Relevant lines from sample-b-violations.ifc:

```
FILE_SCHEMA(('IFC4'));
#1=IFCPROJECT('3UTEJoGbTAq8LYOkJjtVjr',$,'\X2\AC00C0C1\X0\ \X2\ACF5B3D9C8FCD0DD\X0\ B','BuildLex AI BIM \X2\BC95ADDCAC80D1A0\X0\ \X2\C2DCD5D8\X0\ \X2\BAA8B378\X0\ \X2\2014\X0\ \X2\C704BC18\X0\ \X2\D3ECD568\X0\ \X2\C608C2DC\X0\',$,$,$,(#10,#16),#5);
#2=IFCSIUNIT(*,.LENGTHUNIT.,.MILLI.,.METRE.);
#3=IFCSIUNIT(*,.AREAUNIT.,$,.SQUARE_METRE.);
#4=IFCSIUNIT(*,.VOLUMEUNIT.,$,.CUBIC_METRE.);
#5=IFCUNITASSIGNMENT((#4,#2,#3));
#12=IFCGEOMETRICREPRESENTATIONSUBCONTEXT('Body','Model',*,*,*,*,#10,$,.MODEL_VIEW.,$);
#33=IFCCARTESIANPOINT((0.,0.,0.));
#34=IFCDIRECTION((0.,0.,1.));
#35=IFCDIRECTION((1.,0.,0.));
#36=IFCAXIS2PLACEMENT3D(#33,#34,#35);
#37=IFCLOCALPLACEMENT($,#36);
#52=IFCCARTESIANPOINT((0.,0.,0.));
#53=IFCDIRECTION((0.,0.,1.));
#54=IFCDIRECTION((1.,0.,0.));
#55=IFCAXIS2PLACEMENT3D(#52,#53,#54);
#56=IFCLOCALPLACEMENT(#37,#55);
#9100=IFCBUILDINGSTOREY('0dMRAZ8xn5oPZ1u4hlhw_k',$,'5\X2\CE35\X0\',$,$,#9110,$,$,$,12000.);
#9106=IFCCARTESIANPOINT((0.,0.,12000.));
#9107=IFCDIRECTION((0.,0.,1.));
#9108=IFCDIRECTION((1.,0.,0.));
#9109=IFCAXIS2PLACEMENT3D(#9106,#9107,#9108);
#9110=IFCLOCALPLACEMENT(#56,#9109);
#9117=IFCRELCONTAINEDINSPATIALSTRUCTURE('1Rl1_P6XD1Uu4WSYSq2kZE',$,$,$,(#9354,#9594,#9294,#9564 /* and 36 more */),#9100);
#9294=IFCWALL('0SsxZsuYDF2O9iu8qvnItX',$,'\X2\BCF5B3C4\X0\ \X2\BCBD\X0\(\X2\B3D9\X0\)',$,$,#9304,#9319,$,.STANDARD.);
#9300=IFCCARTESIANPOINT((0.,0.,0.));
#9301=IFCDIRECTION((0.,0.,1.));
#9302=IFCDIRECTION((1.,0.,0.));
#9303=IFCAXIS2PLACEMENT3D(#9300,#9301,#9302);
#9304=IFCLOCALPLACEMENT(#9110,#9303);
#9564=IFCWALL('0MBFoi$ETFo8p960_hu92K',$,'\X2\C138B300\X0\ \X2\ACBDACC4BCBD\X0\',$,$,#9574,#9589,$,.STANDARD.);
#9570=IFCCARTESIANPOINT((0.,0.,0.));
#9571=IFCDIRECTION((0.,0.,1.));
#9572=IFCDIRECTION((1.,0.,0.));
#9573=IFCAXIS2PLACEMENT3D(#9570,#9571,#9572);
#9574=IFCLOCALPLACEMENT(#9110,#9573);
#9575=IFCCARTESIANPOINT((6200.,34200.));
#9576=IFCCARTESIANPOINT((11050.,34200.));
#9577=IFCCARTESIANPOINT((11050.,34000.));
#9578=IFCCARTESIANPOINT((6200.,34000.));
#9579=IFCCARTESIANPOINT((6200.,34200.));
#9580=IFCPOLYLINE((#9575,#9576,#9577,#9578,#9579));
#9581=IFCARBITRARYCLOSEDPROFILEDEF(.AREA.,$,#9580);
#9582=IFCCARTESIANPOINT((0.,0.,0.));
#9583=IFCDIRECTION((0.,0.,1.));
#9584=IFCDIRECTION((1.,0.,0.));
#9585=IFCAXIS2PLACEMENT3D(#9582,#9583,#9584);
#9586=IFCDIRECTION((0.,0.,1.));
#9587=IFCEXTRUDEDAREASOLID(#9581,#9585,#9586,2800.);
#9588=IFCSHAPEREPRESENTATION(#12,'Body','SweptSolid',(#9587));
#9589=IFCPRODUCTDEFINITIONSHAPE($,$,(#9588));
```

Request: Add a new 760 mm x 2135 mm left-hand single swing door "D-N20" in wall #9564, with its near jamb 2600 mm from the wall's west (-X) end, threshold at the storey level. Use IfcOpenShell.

```python
import numpy as np
import ifcopenshell
import ifcopenshell.api.feature
import ifcopenshell.api.geometry
import ifcopenshell.api.root
import ifcopenshell.api.spatial
import ifcopenshell.geom
import ifcopenshell.util.element
import ifcopenshell.util.placement
import ifcopenshell.util.representation
import ifcopenshell.util.shape
import ifcopenshell.util.unit

model = ifcopenshell.open("sample-b-violations.ifc")
unit_scale = ifcopenshell.util.unit.calculate_unit_scale(model)
settings = ifcopenshell.geom.settings()


def volume(element):
    """Net volume in cubic metres, openings subtracted."""
    shape = ifcopenshell.geom.create_shape(settings, element)
    return ifcopenshell.util.shape.get_volume(shape.geometry)


wall = model.by_guid("0MBFoi$ETFo8p960_hu92K")
storey = ifcopenshell.util.element.get_container(wall, ifc_class="IfcBuildingStorey")
context = ifcopenshell.util.representation.get_context(model, "Model", "Body", "MODEL_VIEW")
before = volume(wall)

width, height, from_end, sill = 0.76, 2.135, 2.6, 0.0  # metres

# The wall runs along its own X axis, and the end named is its -X end.
wall_shape = ifcopenshell.geom.create_shape(settings, wall)
x, y, z = ifcopenshell.util.shape.get_vertices(wall_shape.geometry).T
start = x.min() + from_end
face, thickness = float(y.min()), float(y.max() - y.min())
wall_matrix = ifcopenshell.util.placement.get_local_placement(wall.ObjectPlacement)
level = ifcopenshell.util.placement.get_local_placement(storey.ObjectPlacement)[2, 3]


def in_wall(x, y):
    """Placement at x, y metres in the wall's axes, at sill height."""
    matrix = wall_matrix.copy()
    matrix[:, 3] = wall_matrix @ np.array([x / unit_scale, y / unit_scale, 0.0, 1.0])
    matrix[2, 3] = level + sill / unit_scale
    return matrix


# Opening: a box that overshoots both wall faces by 50 mm.
opening = ifcopenshell.api.root.create_entity(model, ifc_class="IfcOpeningElement", predefined_type="OPENING")
box = ifcopenshell.api.geometry.add_wall_representation(
    model, context=context, length=width, height=height, thickness=thickness + 0.1
)
ifcopenshell.api.geometry.assign_representation(model, product=opening, representation=box)
ifcopenshell.api.geometry.edit_object_placement(model, product=opening, matrix=in_wall(start, face - 0.05), is_si=False)
ifcopenshell.api.feature.add_feature(model, feature=opening, element=wall)

door = ifcopenshell.api.root.create_entity(model, ifc_class="IfcDoor", name="D-N20", predefined_type="DOOR")
door.OverallWidth, door.OverallHeight = width / unit_scale, height / unit_scale
door.OperationType = "SINGLE_SWING_LEFT"
body = ifcopenshell.api.geometry.add_door_representation(
    model,
    context=context,
    overall_width=door.OverallWidth,
    overall_height=door.OverallHeight,
    operation_type="SINGLE_SWING_LEFT",
    lining_properties={"LiningDepth": thickness / unit_scale, "ThresholdDepth": thickness / unit_scale},
)
ifcopenshell.api.geometry.assign_representation(model, product=door, representation=body)
ifcopenshell.api.spatial.assign_container(model, products=[door], relating_structure=storey)
ifcopenshell.api.feature.add_filling(model, opening=opening, element=door)

# The lining spans the wall, so the door starts at the wall face.
ifcopenshell.api.geometry.edit_object_placement(model, product=door, matrix=in_wall(start, face), is_si=False)

after = volume(wall)

print(f"wall volume {before:.3f} -> {after:.3f} m3")

model.write("sample-b-violations_updated.ifc")
```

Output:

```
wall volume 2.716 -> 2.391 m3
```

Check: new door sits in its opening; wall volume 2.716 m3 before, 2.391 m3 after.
